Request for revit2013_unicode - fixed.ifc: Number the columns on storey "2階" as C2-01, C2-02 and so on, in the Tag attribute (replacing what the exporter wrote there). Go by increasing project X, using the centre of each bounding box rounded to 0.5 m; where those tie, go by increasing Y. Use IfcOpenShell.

First a look at what the model holds.

```python
import ifcopenshell
import ifcopenshell.util.element
import ifcopenshell.util.placement

model = ifcopenshell.open("revit2013_unicode - fixed.ifc")
print(model.schema)
storey = next(s for s in model.by_type("IfcBuildingStorey") if s.Name == "2階")
columns = [e for e in ifcopenshell.util.element.get_decomposition(storey) if e.is_a("IfcColumn")]
for e in sorted(columns, key=lambda e: e.id()):
    origin = ifcopenshell.util.placement.get_local_placement(e.ObjectPlacement)[:3, 3]
    print(e.id(), e.Tag, e.Name, origin.round(2) + 0.0, sep=" | ")
```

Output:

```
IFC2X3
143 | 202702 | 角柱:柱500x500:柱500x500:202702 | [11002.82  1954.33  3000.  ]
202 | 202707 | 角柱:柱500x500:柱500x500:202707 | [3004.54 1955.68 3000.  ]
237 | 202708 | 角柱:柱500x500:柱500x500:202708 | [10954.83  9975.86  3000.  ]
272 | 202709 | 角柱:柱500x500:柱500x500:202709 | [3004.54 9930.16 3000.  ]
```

```python
import ifcopenshell
import ifcopenshell.geom
import ifcopenshell.util.element
import ifcopenshell.util.shape

model = ifcopenshell.open("revit2013_unicode - fixed.ifc")
settings = ifcopenshell.geom.settings()
settings.set("use-world-coords", True)


def centre(element):
    shape = ifcopenshell.geom.create_shape(settings, element)
    return ifcopenshell.util.shape.get_bbox_centroid(shape.geometry)


storey = next(s for s in model.by_type("IfcBuildingStorey") if s.Name == "2階")
columns = [e for e in ifcopenshell.util.element.get_decomposition(storey) if e.is_a("IfcColumn")]

# Insertion points can sit at a corner or the storey origin, so sort by the geometry (in metres).
centres = {e: centre(e) for e in columns}
columns.sort(key=lambda e: (round(centres[e][0] / 0.5), centres[e][1]))

for i, e in enumerate(columns, start=1):
    number = f"C2-{i:02d}"
    e.Tag = number
    print(e.id(), number)

model.write("revit2013_unicode - fixed_edited.ifc")
```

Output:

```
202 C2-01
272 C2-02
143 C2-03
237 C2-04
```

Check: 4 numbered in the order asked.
